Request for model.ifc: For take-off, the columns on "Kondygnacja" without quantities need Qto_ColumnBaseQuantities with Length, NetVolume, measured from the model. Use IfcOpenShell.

First a look at what the model holds.

```python
import ifcopenshell
import ifcopenshell.util.element
import ifcopenshell.util.unit

model = ifcopenshell.open("model.ifc")
print(model.schema)
for unit_type in ("LENGTHUNIT", "AREAUNIT", "VOLUMEUNIT"):
    print(unit_type, ifcopenshell.util.unit.calculate_unit_scale(model, unit_type))
storey = next(s for s in model.by_type("IfcBuildingStorey") if s.Name == "Kondygnacja")
columns = [e for e in ifcopenshell.util.element.get_decomposition(storey) if e.is_a("IfcColumn")]
for e in sorted(columns, key=lambda e: e.id()):
    print(e.id(), e.is_a(), e.Name, list(ifcopenshell.util.element.get_psets(e, qtos_only=True)), sep=" | ")
```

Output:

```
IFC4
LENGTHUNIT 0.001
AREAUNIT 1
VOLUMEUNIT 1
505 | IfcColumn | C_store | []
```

```python
import ifcopenshell
import ifcopenshell.api.pset
import ifcopenshell.geom
import ifcopenshell.util.element
import ifcopenshell.util.shape
import ifcopenshell.util.unit

model = ifcopenshell.open("model.ifc")
unit_scale = ifcopenshell.util.unit.calculate_unit_scale(model)
volume_scale = ifcopenshell.util.unit.calculate_unit_scale(model, "VOLUMEUNIT")
settings = ifcopenshell.geom.settings()

storey = next(s for s in model.by_type("IfcBuildingStorey") if s.Name == "Kondygnacja")
columns = [e for e in ifcopenshell.util.element.get_decomposition(storey) if e.is_a("IfcColumn")]

for e in sorted(columns, key=lambda e: e.id()):
    if ifcopenshell.util.element.get_psets(e, qtos_only=True, should_inherit=False):
        continue
    # Geometry comes back in metres, in the element's own axes.
    shape = ifcopenshell.geom.create_shape(settings, e)
    values = {
        "Length": ifcopenshell.util.shape.get_z(shape.geometry) / unit_scale,
        "NetVolume": ifcopenshell.util.shape.get_volume(shape.geometry) / volume_scale,
    }
    qto = ifcopenshell.api.pset.add_qto(model, product=e, name="Qto_ColumnBaseQuantities")
    ifcopenshell.api.pset.edit_qto(model, qto=qto, properties=values)
    print(e.id(), {k: round(v, 3) for k, v in values.items()})

model.write("model_edited.ifc")
```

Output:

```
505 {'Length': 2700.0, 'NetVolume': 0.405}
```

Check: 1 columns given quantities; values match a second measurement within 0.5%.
